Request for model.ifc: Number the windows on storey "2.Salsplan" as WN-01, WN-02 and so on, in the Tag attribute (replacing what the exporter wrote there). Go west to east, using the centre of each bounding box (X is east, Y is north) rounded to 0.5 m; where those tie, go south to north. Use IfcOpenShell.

First a look at what the model holds.

```python
import ifcopenshell
import ifcopenshell.util.element
import ifcopenshell.util.placement

model = ifcopenshell.open("model.ifc")
print(model.schema)
storey = next(s for s in model.by_type("IfcBuildingStorey") if s.Name == "2.Salsplan")
windows = [e for e in ifcopenshell.util.element.get_decomposition(storey) if e.is_a("IfcWindow")]
for e in sorted(windows, key=lambda e: e.id()):
    origin = ifcopenshell.util.placement.get_local_placement(e.ObjectPlacement)[:3, 3]
    print(e.id(), e.Tag, e.Name, origin.round(2) + 0.0, sep=" | ")
```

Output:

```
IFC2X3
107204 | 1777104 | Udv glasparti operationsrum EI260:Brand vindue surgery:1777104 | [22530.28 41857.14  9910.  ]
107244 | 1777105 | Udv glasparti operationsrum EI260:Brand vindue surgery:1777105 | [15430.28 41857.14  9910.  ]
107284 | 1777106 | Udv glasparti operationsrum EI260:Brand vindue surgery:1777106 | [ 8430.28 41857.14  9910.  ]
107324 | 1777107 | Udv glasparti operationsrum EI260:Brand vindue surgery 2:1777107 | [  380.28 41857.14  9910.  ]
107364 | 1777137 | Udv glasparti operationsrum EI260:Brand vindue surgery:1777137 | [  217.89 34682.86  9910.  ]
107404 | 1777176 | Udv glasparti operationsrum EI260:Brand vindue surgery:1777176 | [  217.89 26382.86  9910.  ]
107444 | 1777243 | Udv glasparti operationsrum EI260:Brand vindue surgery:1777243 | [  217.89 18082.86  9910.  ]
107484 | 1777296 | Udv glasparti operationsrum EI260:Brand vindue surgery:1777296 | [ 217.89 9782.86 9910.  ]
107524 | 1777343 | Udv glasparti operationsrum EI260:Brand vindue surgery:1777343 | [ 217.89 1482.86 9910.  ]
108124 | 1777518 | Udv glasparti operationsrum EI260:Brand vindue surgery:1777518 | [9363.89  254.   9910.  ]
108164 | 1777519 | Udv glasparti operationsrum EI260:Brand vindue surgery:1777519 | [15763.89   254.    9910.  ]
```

```python
import ifcopenshell
import ifcopenshell.geom
import ifcopenshell.util.element
import ifcopenshell.util.shape

model = ifcopenshell.open("model.ifc")
settings = ifcopenshell.geom.settings()
settings.set("use-world-coords", True)


def centre(element):
    shape = ifcopenshell.geom.create_shape(settings, element)
    return ifcopenshell.util.shape.get_bbox_centroid(shape.geometry)


storey = next(s for s in model.by_type("IfcBuildingStorey") if s.Name == "2.Salsplan")
windows = [e for e in ifcopenshell.util.element.get_decomposition(storey) if e.is_a("IfcWindow")]

# Insertion points can sit at a corner or the storey origin, so sort by the geometry (in metres).
centres = {e: centre(e) for e in windows}
windows.sort(key=lambda e: (round(centres[e][0] / 0.5), centres[e][1]))

for i, e in enumerate(windows, start=1):
    number = f"WN-{i:02d}"
    e.Tag = number
    print(e.id(), number)

model.write("model-out.ifc")
```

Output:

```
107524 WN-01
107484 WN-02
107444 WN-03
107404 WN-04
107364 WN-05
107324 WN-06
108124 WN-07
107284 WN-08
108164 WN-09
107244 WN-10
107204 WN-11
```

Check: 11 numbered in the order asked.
